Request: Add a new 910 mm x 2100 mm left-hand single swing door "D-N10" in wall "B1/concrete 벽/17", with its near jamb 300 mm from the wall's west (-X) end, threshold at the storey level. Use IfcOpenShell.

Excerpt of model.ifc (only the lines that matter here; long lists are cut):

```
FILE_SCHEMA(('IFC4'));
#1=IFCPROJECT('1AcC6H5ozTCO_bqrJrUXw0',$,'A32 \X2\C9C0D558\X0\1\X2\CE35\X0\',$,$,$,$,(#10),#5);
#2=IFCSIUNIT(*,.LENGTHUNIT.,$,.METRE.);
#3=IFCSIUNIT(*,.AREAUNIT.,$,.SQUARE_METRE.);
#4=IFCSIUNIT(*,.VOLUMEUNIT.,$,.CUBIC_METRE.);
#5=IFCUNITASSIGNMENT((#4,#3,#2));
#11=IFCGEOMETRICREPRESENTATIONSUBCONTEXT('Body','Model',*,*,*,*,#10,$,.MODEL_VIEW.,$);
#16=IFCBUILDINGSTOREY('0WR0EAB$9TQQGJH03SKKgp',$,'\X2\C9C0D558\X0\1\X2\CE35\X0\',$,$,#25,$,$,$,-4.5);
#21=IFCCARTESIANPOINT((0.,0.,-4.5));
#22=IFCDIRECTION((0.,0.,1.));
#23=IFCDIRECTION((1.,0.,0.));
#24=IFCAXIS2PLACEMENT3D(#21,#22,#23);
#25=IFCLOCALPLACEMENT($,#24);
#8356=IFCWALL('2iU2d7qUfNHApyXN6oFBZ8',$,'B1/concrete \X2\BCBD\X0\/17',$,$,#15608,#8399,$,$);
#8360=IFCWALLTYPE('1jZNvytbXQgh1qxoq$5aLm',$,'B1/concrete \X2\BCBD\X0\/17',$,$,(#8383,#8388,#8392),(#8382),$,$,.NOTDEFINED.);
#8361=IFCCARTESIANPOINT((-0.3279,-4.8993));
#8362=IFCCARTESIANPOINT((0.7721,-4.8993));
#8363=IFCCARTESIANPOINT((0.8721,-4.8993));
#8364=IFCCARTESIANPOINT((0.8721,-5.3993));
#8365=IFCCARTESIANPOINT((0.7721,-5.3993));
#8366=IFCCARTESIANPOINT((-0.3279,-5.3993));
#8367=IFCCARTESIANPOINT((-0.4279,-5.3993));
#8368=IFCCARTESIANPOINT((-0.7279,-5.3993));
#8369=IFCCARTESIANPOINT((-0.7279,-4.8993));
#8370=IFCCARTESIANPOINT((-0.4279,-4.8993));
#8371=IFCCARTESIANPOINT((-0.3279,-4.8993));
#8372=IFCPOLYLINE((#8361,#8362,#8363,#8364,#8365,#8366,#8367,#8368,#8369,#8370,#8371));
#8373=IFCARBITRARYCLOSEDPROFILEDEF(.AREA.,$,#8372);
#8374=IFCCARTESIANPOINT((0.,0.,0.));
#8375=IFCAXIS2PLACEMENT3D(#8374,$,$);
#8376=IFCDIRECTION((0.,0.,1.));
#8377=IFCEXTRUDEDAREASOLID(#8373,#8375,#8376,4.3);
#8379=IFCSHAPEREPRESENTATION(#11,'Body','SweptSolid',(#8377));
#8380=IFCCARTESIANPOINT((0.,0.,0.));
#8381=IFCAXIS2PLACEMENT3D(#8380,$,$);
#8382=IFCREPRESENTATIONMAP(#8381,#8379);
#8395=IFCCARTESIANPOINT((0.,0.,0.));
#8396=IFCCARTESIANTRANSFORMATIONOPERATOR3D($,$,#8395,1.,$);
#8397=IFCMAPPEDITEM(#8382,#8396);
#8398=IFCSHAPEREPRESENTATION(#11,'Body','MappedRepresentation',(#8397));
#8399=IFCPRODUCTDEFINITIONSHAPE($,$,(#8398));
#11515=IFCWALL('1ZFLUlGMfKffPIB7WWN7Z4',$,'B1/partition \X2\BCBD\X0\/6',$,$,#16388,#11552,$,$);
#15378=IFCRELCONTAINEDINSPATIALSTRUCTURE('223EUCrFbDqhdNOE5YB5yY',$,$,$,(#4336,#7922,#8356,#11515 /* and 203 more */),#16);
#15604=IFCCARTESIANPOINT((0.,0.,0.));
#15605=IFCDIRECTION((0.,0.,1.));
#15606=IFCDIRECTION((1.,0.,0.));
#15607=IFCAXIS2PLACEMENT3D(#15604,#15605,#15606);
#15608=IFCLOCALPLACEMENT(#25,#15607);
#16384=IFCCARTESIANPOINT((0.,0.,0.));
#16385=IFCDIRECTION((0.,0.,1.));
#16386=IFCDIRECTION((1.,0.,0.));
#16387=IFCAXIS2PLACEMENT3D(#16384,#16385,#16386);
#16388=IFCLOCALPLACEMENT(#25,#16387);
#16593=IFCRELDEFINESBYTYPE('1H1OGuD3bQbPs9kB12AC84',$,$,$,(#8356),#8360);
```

```python
import numpy as np
import ifcopenshell
import ifcopenshell.api.feature
import ifcopenshell.api.geometry
import ifcopenshell.api.root
import ifcopenshell.api.spatial
import ifcopenshell.geom
import ifcopenshell.util.element
import ifcopenshell.util.placement
import ifcopenshell.util.representation
import ifcopenshell.util.shape
import ifcopenshell.util.unit

model = ifcopenshell.open("model.ifc")
unit_scale = ifcopenshell.util.unit.calculate_unit_scale(model)
settings = ifcopenshell.geom.settings()


def volume(element):
    """Net volume in cubic metres, openings subtracted."""
    shape = ifcopenshell.geom.create_shape(settings, element)
    return ifcopenshell.util.shape.get_volume(shape.geometry)


wall = model.by_guid("2iU2d7qUfNHApyXN6oFBZ8")
storey = ifcopenshell.util.element.get_container(wall, ifc_class="IfcBuildingStorey")
context = ifcopenshell.util.representation.get_context(model, "Model", "Body", "MODEL_VIEW")
before = volume(wall)

width, height, from_end, sill = 0.91, 2.1, 0.3, 0.0  # metres

# The wall runs along its own X axis, and the end named is its -X end.
wall_shape = ifcopenshell.geom.create_shape(settings, wall)
x, y, z = ifcopenshell.util.shape.get_vertices(wall_shape.geometry).T
start = x.min() + from_end
face, thickness = float(y.min()), float(y.max() - y.min())
wall_matrix = ifcopenshell.util.placement.get_local_placement(wall.ObjectPlacement)
level = ifcopenshell.util.placement.get_local_placement(storey.ObjectPlacement)[2, 3]


def in_wall(x, y):
    """Placement at x, y metres in the wall's axes, at sill height."""
    matrix = wall_matrix.copy()
    matrix[:, 3] = wall_matrix @ np.array([x / unit_scale, y / unit_scale, 0.0, 1.0])
    matrix[2, 3] = level + sill / unit_scale
    return matrix


# Opening: a box that overshoots both wall faces by 50 mm.
opening = ifcopenshell.api.root.create_entity(model, ifc_class="IfcOpeningElement", predefined_type="OPENING")
box = ifcopenshell.api.geometry.add_wall_representation(
    model, context=context, length=width, height=height, thickness=thickness + 0.1
)
ifcopenshell.api.geometry.assign_representation(model, product=opening, representation=box)
ifcopenshell.api.geometry.edit_object_placement(model, product=opening, matrix=in_wall(start, face - 0.05), is_si=False)
ifcopenshell.api.feature.add_feature(model, feature=opening, element=wall)

door = ifcopenshell.api.root.create_entity(model, ifc_class="IfcDoor", name="D-N10", predefined_type="DOOR")
door.OverallWidth, door.OverallHeight = width / unit_scale, height / unit_scale
door.OperationType = "SINGLE_SWING_LEFT"
body = ifcopenshell.api.geometry.add_door_representation(
    model,
    context=context,
    overall_width=door.OverallWidth,
    overall_height=door.OverallHeight,
    operation_type="SINGLE_SWING_LEFT",
    lining_properties={"LiningDepth": thickness / unit_scale, "ThresholdDepth": thickness / unit_scale},
)
ifcopenshell.api.geometry.assign_representation(model, product=door, representation=body)
ifcopenshell.api.spatial.assign_container(model, products=[door], relating_structure=storey)
ifcopenshell.api.feature.add_filling(model, opening=opening, element=door)

# The lining spans the wall, so the door starts at the wall face.
ifcopenshell.api.geometry.edit_object_placement(model, product=door, matrix=in_wall(start, face), is_si=False)

after = volume(wall)

print(f"wall volume {before:.3f} -> {after:.3f} m3")

model.write("model-out.ifc")
```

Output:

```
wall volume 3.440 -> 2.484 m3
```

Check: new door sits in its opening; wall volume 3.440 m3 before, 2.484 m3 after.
